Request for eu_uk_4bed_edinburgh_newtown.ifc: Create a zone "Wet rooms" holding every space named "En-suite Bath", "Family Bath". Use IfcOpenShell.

First a look at what the model holds.

```python
import ifcopenshell

model = ifcopenshell.open("eu_uk_4bed_edinburgh_newtown.ifc")
print(model.schema)
seen = {}
for space in model.by_type("IfcSpace"):
    seen[space.LongName] = seen.get(space.LongName, 0) + 1
for name, count in sorted(seen.items(), key=str):
    print(count, "x", name)
print("zones:", [z.Name for z in model.by_type("IfcZone")][:20])
```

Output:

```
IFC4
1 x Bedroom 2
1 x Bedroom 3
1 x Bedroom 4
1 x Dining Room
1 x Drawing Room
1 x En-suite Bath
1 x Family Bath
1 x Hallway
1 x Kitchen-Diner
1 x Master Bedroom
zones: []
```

```python
import ifcopenshell
import ifcopenshell.api.group
import ifcopenshell.api.root

model = ifcopenshell.open("eu_uk_4bed_edinburgh_newtown.ifc")

names = {"En-suite Bath", "Family Bath"}
spaces = [s for s in model.by_type("IfcSpace") if s.LongName in names]

zone = ifcopenshell.api.root.create_entity(model, ifc_class="IfcZone", name="Wet rooms")
ifcopenshell.api.group.assign_group(model, products=spaces, group=zone)
print(len(spaces), "spaces in", zone.Name)

model.write("eu_uk_4bed_edinburgh_newtown_rev.ifc")
```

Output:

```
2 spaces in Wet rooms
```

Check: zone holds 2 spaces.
